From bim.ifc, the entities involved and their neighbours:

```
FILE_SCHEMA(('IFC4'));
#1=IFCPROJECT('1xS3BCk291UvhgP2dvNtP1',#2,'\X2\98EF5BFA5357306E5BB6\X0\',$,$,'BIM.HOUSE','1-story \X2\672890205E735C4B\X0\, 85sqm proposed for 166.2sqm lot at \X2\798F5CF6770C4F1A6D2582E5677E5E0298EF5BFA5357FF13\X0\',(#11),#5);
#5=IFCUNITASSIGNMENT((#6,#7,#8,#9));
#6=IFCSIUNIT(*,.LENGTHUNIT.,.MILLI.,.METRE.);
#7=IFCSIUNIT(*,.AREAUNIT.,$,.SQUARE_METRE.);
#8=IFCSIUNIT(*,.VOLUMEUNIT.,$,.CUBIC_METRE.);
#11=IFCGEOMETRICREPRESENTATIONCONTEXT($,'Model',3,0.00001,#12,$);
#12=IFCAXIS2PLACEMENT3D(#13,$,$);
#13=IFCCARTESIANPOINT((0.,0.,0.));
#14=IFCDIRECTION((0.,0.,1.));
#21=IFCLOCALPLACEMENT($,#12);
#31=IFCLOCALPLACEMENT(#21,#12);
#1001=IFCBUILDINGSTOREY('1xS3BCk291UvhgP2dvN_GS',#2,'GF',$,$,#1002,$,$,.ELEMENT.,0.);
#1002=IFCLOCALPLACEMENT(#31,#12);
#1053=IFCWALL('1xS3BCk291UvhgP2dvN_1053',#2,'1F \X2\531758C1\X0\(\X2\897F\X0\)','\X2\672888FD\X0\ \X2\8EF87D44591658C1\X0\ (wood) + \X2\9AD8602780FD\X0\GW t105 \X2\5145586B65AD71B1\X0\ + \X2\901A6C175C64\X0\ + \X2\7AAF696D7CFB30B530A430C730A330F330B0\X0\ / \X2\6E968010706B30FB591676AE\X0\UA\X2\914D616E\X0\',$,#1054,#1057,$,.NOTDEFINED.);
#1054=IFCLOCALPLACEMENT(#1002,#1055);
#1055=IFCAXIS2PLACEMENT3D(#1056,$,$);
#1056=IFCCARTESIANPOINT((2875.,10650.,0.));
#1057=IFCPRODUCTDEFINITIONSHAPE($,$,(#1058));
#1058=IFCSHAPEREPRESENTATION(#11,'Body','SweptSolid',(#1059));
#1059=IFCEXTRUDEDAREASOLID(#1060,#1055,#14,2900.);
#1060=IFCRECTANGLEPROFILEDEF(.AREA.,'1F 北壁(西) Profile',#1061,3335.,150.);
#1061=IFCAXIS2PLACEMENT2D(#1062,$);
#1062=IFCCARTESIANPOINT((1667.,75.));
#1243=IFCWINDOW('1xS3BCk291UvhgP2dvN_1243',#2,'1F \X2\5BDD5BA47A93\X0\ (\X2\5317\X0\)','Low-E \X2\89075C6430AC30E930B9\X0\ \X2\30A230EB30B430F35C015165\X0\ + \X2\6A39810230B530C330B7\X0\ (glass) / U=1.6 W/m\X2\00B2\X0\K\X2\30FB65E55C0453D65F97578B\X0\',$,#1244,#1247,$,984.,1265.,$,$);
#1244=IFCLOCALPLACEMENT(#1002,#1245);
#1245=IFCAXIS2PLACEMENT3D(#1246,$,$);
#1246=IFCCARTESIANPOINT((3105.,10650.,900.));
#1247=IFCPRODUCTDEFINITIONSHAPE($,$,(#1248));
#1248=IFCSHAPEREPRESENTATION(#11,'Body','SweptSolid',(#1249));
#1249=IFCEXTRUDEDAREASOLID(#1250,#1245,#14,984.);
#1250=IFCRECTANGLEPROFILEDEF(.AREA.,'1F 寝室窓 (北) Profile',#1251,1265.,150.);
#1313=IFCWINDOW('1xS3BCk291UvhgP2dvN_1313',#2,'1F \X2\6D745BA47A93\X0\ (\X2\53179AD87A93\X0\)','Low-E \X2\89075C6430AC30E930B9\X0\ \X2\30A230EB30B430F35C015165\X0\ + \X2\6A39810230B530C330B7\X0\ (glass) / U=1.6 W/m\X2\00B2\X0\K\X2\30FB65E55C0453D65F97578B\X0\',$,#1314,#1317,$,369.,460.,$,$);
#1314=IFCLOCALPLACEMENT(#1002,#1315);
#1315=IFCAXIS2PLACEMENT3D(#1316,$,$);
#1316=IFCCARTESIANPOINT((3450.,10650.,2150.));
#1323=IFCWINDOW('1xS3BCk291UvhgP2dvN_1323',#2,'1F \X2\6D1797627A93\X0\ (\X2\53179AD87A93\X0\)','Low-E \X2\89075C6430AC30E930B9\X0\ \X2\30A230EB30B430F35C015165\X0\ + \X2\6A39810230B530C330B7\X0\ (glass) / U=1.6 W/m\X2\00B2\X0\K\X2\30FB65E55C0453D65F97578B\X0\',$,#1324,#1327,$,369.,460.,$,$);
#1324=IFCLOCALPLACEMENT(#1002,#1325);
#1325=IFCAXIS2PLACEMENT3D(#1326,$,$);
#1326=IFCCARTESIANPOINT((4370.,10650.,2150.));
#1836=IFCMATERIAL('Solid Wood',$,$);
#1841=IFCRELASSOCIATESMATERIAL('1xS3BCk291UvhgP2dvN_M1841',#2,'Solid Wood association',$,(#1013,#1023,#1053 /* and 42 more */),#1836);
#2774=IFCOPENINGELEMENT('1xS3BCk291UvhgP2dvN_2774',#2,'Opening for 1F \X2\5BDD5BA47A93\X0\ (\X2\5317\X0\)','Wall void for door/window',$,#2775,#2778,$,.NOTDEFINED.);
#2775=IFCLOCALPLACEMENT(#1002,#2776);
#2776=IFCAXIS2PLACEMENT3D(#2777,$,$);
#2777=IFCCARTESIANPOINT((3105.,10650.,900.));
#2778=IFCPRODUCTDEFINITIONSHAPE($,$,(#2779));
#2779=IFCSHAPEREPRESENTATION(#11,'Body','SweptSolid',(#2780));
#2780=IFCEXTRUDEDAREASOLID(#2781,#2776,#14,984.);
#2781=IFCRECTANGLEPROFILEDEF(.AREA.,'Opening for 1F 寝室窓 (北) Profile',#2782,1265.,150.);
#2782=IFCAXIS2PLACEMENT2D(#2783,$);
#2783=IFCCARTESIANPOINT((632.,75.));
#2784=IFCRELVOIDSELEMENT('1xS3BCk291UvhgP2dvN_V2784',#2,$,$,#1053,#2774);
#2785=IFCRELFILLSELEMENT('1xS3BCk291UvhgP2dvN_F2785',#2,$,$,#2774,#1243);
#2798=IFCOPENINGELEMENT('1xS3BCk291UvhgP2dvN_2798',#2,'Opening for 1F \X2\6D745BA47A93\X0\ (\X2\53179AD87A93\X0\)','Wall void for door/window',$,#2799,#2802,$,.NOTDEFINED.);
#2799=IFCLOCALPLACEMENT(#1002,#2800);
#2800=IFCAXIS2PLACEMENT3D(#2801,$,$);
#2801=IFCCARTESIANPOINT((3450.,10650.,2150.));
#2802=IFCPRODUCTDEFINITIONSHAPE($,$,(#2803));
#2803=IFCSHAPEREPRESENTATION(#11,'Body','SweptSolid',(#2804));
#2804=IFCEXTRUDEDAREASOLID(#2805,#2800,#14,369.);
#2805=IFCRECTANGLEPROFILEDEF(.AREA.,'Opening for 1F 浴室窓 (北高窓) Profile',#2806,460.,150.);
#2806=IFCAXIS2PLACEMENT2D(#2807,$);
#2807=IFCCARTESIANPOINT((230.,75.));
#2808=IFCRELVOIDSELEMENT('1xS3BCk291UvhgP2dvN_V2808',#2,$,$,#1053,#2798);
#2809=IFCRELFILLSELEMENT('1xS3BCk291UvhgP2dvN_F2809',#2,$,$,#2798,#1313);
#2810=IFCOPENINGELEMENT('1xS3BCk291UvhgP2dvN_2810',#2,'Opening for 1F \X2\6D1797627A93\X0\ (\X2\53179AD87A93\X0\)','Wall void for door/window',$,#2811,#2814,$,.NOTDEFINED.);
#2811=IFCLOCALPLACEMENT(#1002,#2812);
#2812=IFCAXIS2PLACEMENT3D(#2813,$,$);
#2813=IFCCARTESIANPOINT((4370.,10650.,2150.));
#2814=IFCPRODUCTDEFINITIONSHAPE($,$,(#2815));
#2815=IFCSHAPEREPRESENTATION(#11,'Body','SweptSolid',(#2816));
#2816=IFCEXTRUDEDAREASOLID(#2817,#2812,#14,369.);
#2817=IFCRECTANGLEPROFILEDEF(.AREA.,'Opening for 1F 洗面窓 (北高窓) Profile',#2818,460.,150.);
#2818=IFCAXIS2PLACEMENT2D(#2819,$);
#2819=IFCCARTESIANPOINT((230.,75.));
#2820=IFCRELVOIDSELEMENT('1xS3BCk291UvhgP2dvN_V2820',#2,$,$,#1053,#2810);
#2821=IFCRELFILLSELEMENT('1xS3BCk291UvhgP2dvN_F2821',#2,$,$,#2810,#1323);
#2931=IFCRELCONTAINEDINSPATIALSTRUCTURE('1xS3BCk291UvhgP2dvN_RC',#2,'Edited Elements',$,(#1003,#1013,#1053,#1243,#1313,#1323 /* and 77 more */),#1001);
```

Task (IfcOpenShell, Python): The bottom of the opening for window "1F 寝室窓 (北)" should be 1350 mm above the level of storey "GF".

```python
import numpy as np
import ifcopenshell
import ifcopenshell.api.geometry
import ifcopenshell.geom
import ifcopenshell.util.element
import ifcopenshell.util.placement
import ifcopenshell.util.shape
import ifcopenshell.util.unit

model = ifcopenshell.open("bim.ifc")
unit_scale = ifcopenshell.util.unit.calculate_unit_scale(model)

window = model.by_guid("1xS3BCk291UvhgP2dvN_1243")
opening = window.FillsVoids[0].RelatingOpeningElement
storey = ifcopenshell.util.element.get_container(window, ifc_class="IfcBuildingStorey")
level = ifcopenshell.util.placement.get_local_placement(storey.ObjectPlacement)[2, 3]

# The opening's origin need not be at the sill, so measure its lowest point.
shape = ifcopenshell.geom.create_shape(ifcopenshell.geom.settings(), opening)
bottom = ifcopenshell.util.shape.get_shape_bottom_elevation(shape, shape.geometry) / unit_scale
dz = level + 1350.0 - bottom

shift = np.array([0.0, 0.0, dz])
# The window is not placed relative to its opening, so move both.
for product in (opening, window):
    matrix = ifcopenshell.util.placement.get_local_placement(product.ObjectPlacement)
    matrix[:3, 3] += shift
    ifcopenshell.api.geometry.edit_object_placement(model, product=product, matrix=matrix, is_si=False)

print(f"moved by {dz * unit_scale:+.3f} m")

model.write("bim_v2.ifc")
```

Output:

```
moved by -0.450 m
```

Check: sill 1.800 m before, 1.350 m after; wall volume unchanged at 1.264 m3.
